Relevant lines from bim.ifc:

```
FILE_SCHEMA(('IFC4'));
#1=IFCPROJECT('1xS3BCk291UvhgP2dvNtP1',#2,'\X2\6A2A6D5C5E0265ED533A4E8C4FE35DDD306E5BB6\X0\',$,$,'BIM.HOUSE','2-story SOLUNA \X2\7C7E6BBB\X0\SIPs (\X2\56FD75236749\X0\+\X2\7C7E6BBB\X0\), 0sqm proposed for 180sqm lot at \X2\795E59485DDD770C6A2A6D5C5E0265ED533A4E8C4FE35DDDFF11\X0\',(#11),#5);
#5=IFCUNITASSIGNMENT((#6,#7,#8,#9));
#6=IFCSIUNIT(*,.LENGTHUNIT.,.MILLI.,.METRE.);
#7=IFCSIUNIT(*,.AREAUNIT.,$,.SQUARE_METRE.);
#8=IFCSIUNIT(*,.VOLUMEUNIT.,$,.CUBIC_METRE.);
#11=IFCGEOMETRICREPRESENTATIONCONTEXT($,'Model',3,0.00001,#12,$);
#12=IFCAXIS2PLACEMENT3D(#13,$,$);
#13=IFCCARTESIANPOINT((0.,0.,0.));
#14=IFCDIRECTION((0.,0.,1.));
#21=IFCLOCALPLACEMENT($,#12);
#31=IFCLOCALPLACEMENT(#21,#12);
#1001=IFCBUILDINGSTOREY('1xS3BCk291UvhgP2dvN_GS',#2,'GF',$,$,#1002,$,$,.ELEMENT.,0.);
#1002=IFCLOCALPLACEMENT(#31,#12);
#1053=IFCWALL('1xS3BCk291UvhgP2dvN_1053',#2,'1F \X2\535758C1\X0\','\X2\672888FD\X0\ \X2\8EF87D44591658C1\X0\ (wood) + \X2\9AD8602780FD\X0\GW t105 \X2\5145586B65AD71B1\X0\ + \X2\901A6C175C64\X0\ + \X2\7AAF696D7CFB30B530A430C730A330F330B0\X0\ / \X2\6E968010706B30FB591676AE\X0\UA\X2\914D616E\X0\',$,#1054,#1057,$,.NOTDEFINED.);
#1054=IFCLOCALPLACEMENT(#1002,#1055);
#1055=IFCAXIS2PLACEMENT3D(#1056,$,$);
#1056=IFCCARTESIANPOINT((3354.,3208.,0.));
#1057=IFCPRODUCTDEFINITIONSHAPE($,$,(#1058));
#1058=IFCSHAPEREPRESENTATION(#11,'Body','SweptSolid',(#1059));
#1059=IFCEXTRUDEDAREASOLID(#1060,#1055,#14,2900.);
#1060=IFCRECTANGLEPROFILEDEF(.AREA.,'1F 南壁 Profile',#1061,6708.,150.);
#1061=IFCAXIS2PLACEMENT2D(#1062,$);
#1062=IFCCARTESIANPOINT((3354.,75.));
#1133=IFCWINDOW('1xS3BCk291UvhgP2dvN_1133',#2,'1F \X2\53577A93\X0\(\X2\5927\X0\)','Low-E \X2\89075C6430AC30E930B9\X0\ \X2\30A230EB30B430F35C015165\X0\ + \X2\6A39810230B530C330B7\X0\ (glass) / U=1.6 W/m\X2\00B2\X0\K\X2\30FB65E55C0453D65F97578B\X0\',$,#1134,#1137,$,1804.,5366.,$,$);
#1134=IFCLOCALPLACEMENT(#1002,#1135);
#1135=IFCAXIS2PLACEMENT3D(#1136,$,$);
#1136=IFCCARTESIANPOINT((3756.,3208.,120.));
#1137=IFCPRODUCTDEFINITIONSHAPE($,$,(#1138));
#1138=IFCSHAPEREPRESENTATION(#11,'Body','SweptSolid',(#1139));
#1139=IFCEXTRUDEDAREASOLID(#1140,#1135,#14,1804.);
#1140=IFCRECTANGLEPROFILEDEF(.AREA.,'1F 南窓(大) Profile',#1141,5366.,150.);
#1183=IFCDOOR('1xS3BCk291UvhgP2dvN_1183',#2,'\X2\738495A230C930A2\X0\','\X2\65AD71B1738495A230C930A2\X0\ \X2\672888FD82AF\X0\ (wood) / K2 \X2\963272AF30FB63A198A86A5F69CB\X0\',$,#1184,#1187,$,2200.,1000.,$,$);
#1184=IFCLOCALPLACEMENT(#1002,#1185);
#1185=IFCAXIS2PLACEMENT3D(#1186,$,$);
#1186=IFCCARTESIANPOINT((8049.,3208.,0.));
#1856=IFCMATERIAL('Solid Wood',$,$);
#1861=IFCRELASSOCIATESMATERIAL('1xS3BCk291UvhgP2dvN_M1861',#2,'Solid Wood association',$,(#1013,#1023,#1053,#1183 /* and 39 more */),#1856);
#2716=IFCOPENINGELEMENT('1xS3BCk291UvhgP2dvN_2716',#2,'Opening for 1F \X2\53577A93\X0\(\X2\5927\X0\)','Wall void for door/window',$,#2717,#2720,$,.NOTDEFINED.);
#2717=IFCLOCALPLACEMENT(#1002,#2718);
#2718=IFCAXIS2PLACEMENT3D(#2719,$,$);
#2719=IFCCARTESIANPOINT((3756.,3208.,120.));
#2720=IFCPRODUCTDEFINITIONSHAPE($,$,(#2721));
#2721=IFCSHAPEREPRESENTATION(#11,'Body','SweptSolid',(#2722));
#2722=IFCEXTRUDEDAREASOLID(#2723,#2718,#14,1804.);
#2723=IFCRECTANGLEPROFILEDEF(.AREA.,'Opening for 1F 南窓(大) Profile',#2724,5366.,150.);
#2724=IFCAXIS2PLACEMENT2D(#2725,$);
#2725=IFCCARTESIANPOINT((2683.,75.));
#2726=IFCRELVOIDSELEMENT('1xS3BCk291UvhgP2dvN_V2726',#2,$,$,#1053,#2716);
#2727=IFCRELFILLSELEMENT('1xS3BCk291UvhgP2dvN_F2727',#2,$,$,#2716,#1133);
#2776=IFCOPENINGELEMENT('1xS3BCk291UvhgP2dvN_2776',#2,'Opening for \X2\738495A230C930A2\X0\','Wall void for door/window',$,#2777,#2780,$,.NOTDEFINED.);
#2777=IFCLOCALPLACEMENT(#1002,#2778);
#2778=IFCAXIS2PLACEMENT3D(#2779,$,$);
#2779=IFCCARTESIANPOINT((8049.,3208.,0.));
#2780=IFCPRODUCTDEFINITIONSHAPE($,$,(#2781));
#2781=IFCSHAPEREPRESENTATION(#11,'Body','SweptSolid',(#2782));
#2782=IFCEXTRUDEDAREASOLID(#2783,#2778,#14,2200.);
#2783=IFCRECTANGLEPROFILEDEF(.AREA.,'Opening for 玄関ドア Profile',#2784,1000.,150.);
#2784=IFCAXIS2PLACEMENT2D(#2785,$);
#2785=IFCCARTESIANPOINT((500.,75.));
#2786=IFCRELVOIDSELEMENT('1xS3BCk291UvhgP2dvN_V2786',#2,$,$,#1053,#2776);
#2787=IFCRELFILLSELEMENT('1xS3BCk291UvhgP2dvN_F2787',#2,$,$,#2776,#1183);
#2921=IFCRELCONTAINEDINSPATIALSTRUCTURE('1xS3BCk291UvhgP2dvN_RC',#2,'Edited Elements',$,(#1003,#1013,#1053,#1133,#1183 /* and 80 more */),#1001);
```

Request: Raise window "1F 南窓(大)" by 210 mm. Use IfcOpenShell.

```python
import numpy as np
import ifcopenshell
import ifcopenshell.api.geometry
import ifcopenshell.util.placement
import ifcopenshell.util.unit

model = ifcopenshell.open("bim.ifc")
unit_scale = ifcopenshell.util.unit.calculate_unit_scale(model)

window = model.by_guid("1xS3BCk291UvhgP2dvN_1133")
opening = window.FillsVoids[0].RelatingOpeningElement
dz = 210.0

shift = np.array([0.0, 0.0, dz])
# The window is not placed relative to its opening, so move both.
for product in (opening, window):
    matrix = ifcopenshell.util.placement.get_local_placement(product.ObjectPlacement)
    matrix[:3, 3] += shift
    ifcopenshell.api.geometry.edit_object_placement(model, product=product, matrix=matrix, is_si=False)

print(f"moved by {dz * unit_scale:+.3f} m")

model.write("bim_v2.ifc")
```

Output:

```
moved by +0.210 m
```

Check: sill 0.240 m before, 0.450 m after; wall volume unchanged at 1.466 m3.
